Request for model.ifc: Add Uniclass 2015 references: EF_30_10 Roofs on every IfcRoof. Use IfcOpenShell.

First a look at what the model holds.

```python
import ifcopenshell

model = ifcopenshell.open("model.ifc")
print(model.schema)
print("classifications:", [c.Name for c in model.by_type("IfcClassification")])
for ifc_class in ("IfcDoor", "IfcRoof", "IfcStair", "IfcWall", "IfcWindow"):
    print(ifc_class, len(model.by_type(ifc_class)))
```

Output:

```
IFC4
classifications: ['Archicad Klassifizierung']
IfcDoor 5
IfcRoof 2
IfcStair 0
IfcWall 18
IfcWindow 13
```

```python
import ifcopenshell
import ifcopenshell.api.classification

model = ifcopenshell.open("model.ifc")

system = ifcopenshell.api.classification.add_classification(model, classification="Uniclass 2015")

codes = {
    "IfcRoof": ("EF_30_10", "Roofs"),
}
for ifc_class, (code, name) in codes.items():
    products = model.by_type(ifc_class)
    ifcopenshell.api.classification.add_reference(
        model, products=products, classification=system, identification=code, name=name
    )
    print(code, len(products))

model.write("model_v2.ifc")
```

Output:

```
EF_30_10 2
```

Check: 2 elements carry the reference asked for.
